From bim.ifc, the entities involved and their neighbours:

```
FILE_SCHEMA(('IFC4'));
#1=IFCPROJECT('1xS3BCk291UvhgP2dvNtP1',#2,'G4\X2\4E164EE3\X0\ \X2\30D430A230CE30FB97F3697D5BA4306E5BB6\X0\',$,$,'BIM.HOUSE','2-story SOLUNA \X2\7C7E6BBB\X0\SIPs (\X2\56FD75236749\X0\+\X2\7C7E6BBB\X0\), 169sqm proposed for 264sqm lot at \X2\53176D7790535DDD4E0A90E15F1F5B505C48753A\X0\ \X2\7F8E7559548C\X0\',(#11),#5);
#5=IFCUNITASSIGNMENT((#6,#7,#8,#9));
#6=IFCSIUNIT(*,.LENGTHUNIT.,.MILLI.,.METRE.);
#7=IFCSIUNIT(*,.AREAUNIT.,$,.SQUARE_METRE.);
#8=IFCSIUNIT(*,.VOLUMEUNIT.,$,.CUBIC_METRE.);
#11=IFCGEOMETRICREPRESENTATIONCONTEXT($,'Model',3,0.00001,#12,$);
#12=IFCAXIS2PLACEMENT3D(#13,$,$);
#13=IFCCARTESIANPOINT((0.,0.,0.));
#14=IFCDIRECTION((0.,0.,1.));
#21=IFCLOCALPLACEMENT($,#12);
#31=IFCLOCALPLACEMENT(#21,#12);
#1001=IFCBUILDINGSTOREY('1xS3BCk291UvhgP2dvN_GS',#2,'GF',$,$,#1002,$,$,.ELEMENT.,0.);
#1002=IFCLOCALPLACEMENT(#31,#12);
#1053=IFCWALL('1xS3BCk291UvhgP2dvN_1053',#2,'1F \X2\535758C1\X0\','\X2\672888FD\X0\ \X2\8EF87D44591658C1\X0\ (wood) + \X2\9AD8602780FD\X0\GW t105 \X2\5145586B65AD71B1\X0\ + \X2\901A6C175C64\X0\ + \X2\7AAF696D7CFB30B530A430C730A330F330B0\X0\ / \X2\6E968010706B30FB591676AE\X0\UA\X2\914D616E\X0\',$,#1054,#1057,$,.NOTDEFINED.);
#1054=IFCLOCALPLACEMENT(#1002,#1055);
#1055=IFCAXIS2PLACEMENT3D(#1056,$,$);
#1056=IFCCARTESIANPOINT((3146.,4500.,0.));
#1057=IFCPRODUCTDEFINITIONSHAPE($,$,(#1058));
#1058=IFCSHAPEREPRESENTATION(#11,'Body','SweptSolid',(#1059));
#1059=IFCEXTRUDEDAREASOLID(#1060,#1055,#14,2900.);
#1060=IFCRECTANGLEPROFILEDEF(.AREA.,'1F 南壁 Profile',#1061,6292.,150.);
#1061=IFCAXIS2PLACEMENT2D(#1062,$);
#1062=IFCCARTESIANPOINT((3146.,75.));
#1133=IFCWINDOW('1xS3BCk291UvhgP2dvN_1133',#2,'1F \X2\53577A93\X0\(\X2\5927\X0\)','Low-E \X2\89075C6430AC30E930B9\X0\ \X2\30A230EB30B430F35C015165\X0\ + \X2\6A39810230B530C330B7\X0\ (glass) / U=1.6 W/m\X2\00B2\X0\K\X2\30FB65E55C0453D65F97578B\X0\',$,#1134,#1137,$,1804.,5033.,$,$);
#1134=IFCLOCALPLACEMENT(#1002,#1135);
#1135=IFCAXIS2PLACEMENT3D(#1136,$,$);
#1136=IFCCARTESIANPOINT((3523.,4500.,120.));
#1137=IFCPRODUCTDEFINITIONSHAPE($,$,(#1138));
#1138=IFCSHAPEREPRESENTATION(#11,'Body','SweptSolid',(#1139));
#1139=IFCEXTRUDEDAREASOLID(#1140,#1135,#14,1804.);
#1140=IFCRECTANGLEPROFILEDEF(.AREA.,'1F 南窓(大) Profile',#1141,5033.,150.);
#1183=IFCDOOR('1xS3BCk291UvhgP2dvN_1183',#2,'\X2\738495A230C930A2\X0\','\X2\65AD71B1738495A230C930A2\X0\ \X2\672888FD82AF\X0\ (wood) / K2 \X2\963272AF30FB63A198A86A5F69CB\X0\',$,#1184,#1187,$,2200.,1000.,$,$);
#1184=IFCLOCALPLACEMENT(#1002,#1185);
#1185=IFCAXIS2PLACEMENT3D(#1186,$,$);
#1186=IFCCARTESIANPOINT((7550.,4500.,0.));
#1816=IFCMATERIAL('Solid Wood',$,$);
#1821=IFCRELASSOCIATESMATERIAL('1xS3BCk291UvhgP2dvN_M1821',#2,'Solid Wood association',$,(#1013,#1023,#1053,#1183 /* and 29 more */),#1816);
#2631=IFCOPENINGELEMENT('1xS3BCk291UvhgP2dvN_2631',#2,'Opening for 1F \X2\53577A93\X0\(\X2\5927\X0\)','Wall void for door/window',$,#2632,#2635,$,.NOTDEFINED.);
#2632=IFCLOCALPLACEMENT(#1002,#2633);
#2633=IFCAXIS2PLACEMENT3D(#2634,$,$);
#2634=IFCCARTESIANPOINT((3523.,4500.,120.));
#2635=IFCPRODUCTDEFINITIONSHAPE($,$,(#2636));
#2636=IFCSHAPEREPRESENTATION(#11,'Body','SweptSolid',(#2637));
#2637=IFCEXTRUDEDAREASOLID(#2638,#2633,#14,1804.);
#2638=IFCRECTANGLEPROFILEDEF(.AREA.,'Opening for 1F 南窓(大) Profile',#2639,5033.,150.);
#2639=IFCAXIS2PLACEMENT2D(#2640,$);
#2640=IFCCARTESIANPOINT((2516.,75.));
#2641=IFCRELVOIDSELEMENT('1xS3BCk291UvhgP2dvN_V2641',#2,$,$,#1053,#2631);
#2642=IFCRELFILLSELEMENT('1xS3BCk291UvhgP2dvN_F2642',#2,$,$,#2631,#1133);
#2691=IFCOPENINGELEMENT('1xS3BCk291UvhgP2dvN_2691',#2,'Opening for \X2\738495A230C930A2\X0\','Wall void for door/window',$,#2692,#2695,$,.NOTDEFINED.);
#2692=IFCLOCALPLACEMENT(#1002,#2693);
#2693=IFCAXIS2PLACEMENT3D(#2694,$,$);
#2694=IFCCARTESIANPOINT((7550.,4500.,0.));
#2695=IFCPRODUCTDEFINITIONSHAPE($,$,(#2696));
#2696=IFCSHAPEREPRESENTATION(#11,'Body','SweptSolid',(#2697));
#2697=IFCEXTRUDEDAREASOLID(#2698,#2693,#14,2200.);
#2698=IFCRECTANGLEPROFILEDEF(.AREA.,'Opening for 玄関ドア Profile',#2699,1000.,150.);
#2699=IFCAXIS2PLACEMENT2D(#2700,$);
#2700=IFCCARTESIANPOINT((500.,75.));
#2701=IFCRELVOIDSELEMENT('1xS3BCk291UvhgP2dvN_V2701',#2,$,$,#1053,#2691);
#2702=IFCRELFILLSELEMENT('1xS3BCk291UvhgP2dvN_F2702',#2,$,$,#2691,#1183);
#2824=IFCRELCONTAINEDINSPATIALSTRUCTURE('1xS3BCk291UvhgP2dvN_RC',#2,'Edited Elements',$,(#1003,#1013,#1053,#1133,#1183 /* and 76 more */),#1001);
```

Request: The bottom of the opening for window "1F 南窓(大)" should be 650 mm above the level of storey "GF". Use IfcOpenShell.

```python
import numpy as np
import ifcopenshell
import ifcopenshell.api.geometry
import ifcopenshell.geom
import ifcopenshell.util.element
import ifcopenshell.util.placement
import ifcopenshell.util.shape
import ifcopenshell.util.unit

model = ifcopenshell.open("bim.ifc")
unit_scale = ifcopenshell.util.unit.calculate_unit_scale(model)

window = model.by_guid("1xS3BCk291UvhgP2dvN_1133")
opening = window.FillsVoids[0].RelatingOpeningElement
storey = ifcopenshell.util.element.get_container(window, ifc_class="IfcBuildingStorey")
level = ifcopenshell.util.placement.get_local_placement(storey.ObjectPlacement)[2, 3]

# The opening's origin need not be at the sill, so measure its lowest point.
shape = ifcopenshell.geom.create_shape(ifcopenshell.geom.settings(), opening)
bottom = ifcopenshell.util.shape.get_shape_bottom_elevation(shape, shape.geometry) / unit_scale
dz = level + 0.65 / unit_scale - bottom

shift = np.array([0.0, 0.0, dz])
# The window is not placed relative to its opening, so move both.
for product in (opening, window):
    matrix = ifcopenshell.util.placement.get_local_placement(product.ObjectPlacement)
    matrix[:3, 3] += shift
    ifcopenshell.api.geometry.edit_object_placement(model, product=product, matrix=matrix, is_si=False)

print(f"moved by {dz * unit_scale:+.3f} m")

model.write("bim_v2.ifc")
```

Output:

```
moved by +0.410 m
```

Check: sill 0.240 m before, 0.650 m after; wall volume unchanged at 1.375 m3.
